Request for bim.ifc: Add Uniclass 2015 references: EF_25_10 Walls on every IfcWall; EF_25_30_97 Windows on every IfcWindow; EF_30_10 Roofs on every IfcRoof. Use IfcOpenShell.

First a look at what the model holds.

```python
import ifcopenshell

model = ifcopenshell.open("bim.ifc")
print(model.schema)
print("classifications:", [c.Name for c in model.by_type("IfcClassification")])
for ifc_class in ("IfcDoor", "IfcRoof", "IfcStair", "IfcWall", "IfcWindow"):
    print(ifc_class, len(model.by_type(ifc_class)))
```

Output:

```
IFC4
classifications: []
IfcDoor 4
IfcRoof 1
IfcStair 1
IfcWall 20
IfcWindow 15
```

```python
import ifcopenshell
import ifcopenshell.api.classification

model = ifcopenshell.open("bim.ifc")

system = ifcopenshell.api.classification.add_classification(model, classification="Uniclass 2015")

codes = {
    "IfcWall": ("EF_25_10", "Walls"),
    "IfcWindow": ("EF_25_30_97", "Windows"),
    "IfcRoof": ("EF_30_10", "Roofs"),
}
for ifc_class, (code, name) in codes.items():
    products = model.by_type(ifc_class)
    ifcopenshell.api.classification.add_reference(
        model, products=products, classification=system, identification=code, name=name
    )
    print(code, len(products))

model.write("bim_updated.ifc")
```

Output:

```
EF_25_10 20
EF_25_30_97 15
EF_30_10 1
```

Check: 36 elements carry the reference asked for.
